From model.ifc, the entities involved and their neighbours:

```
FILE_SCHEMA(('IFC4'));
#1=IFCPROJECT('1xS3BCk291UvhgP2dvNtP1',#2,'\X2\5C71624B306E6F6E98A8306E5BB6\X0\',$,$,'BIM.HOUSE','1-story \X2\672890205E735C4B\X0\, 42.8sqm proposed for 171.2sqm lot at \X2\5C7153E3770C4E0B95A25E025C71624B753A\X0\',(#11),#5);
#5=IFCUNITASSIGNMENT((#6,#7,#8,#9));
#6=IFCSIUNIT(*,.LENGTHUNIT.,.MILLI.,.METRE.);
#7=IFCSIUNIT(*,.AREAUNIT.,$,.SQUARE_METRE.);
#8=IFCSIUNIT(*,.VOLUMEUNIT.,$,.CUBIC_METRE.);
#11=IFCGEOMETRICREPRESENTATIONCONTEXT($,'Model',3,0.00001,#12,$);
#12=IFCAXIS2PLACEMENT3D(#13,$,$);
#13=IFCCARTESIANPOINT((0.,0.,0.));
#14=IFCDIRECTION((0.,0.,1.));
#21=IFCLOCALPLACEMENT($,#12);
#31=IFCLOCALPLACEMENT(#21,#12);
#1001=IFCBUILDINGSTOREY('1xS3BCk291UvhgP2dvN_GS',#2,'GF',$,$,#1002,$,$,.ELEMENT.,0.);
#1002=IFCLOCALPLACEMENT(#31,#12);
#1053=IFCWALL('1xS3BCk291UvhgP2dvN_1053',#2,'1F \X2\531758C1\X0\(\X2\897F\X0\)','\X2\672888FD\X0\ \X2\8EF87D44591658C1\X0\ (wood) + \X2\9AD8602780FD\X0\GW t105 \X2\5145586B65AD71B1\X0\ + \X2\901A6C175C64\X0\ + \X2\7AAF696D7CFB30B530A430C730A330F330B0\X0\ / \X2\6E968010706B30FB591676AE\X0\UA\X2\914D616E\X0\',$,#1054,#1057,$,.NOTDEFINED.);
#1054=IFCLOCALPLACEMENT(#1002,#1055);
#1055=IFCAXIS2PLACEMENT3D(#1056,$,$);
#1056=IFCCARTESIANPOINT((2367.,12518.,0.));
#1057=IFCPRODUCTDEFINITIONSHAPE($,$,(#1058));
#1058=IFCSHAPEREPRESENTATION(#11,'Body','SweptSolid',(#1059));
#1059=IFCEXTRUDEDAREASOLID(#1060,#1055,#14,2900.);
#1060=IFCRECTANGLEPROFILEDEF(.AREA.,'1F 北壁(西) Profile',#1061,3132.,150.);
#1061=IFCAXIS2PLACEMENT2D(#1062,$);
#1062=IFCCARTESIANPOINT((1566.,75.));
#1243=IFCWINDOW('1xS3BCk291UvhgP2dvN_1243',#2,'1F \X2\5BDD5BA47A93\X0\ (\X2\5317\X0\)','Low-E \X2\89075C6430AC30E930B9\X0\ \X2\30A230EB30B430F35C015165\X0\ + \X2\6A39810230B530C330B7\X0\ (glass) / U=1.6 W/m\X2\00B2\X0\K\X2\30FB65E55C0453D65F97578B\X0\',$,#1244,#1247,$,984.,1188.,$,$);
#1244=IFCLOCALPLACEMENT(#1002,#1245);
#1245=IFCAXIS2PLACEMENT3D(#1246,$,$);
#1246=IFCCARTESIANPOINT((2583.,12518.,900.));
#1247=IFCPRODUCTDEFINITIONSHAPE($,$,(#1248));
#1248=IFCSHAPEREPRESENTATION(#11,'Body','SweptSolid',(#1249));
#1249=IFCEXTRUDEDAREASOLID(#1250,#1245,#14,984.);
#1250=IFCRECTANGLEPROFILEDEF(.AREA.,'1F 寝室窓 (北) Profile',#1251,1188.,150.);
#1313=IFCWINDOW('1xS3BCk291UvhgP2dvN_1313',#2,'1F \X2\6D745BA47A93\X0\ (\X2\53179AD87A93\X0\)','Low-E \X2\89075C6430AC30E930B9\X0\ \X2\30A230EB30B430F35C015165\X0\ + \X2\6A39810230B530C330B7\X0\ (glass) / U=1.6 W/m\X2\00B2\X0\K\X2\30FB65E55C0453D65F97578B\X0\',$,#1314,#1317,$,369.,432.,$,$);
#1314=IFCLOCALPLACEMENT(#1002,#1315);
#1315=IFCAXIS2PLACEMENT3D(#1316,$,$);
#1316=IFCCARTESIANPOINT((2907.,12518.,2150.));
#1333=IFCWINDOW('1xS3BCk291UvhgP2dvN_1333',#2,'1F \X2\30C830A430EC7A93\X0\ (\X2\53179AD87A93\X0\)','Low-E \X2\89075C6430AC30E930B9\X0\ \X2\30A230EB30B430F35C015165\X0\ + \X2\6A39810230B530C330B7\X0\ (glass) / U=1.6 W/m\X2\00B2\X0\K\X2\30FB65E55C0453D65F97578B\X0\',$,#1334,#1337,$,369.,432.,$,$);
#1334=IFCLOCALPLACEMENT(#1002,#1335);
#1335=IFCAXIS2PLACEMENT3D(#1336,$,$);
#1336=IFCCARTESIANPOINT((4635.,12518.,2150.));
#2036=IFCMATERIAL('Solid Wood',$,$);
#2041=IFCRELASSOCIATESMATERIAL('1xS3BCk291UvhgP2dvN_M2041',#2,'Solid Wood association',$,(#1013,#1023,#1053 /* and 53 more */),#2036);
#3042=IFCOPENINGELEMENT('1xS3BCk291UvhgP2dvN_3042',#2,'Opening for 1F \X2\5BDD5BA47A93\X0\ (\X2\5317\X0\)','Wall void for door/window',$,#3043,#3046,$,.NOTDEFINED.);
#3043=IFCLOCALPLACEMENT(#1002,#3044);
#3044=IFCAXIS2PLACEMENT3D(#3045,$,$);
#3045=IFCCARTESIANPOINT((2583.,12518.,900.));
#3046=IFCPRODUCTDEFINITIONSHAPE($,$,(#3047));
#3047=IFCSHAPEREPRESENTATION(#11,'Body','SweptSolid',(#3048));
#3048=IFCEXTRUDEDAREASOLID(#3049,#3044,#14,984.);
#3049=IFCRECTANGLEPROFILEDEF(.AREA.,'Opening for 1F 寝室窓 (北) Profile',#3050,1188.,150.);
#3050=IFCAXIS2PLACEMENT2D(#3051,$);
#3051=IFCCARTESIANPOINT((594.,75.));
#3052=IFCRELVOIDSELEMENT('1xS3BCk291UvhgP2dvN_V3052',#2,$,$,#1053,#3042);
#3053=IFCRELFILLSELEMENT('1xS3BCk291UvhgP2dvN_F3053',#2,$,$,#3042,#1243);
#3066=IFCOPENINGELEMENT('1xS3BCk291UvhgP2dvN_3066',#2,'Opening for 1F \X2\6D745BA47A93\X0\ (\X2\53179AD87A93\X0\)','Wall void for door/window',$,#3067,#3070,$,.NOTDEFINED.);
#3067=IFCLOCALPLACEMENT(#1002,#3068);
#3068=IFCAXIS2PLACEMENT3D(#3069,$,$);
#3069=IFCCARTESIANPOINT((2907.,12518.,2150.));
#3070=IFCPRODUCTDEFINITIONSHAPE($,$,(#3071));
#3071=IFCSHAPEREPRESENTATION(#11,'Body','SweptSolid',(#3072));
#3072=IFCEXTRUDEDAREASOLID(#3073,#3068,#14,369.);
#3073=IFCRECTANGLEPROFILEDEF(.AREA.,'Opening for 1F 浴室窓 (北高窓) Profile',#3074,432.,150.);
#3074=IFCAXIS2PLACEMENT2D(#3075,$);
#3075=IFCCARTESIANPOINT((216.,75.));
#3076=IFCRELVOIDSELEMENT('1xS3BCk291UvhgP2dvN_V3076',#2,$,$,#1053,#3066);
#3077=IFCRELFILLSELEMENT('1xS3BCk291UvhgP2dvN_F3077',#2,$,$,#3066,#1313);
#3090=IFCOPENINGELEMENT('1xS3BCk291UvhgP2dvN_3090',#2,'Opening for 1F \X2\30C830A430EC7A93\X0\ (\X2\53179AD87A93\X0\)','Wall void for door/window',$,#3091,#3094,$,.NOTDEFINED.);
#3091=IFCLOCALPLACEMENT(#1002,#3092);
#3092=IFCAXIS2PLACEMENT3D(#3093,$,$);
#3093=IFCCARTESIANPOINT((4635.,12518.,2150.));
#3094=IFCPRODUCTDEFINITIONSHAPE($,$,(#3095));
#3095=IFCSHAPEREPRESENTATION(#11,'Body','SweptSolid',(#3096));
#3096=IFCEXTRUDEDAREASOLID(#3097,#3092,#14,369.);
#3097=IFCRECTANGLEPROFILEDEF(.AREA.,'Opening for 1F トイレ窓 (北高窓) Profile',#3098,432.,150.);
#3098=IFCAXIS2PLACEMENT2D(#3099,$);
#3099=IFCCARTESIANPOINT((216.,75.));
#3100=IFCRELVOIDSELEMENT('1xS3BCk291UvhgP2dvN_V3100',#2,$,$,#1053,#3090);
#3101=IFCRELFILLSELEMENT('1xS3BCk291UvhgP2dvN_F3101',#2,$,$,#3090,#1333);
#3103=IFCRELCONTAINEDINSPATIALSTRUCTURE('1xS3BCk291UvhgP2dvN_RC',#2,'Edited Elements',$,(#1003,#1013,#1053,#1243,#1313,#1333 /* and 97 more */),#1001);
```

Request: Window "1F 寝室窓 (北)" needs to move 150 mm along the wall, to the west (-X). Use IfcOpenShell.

```python
import ifcopenshell
import ifcopenshell.api.geometry
import ifcopenshell.util.placement

model = ifcopenshell.open("model.ifc")

window = model.by_guid("1xS3BCk291UvhgP2dvN_1243")
opening = window.FillsVoids[0].RelatingOpeningElement
wall = opening.VoidsElements[0].RelatingBuildingElement

wall_matrix = ifcopenshell.util.placement.get_local_placement(wall.ObjectPlacement)
shift = wall_matrix[:3, 0] * -150.0
before = ifcopenshell.util.placement.get_local_placement(window.ObjectPlacement)[:3, 3].copy()

# The window is not placed relative to its opening, so move both.
for product in (opening, window):
    matrix = ifcopenshell.util.placement.get_local_placement(product.ObjectPlacement)
    matrix[:3, 3] += shift
    ifcopenshell.api.geometry.edit_object_placement(model, product=product, matrix=matrix, is_si=False)

after = ifcopenshell.util.placement.get_local_placement(window.ObjectPlacement)[:3, 3]
print("window moved by", (after - before).round(3) + 0.0)

model.write("model_updated.ifc")
```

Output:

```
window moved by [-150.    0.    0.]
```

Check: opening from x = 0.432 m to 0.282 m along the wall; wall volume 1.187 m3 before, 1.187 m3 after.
